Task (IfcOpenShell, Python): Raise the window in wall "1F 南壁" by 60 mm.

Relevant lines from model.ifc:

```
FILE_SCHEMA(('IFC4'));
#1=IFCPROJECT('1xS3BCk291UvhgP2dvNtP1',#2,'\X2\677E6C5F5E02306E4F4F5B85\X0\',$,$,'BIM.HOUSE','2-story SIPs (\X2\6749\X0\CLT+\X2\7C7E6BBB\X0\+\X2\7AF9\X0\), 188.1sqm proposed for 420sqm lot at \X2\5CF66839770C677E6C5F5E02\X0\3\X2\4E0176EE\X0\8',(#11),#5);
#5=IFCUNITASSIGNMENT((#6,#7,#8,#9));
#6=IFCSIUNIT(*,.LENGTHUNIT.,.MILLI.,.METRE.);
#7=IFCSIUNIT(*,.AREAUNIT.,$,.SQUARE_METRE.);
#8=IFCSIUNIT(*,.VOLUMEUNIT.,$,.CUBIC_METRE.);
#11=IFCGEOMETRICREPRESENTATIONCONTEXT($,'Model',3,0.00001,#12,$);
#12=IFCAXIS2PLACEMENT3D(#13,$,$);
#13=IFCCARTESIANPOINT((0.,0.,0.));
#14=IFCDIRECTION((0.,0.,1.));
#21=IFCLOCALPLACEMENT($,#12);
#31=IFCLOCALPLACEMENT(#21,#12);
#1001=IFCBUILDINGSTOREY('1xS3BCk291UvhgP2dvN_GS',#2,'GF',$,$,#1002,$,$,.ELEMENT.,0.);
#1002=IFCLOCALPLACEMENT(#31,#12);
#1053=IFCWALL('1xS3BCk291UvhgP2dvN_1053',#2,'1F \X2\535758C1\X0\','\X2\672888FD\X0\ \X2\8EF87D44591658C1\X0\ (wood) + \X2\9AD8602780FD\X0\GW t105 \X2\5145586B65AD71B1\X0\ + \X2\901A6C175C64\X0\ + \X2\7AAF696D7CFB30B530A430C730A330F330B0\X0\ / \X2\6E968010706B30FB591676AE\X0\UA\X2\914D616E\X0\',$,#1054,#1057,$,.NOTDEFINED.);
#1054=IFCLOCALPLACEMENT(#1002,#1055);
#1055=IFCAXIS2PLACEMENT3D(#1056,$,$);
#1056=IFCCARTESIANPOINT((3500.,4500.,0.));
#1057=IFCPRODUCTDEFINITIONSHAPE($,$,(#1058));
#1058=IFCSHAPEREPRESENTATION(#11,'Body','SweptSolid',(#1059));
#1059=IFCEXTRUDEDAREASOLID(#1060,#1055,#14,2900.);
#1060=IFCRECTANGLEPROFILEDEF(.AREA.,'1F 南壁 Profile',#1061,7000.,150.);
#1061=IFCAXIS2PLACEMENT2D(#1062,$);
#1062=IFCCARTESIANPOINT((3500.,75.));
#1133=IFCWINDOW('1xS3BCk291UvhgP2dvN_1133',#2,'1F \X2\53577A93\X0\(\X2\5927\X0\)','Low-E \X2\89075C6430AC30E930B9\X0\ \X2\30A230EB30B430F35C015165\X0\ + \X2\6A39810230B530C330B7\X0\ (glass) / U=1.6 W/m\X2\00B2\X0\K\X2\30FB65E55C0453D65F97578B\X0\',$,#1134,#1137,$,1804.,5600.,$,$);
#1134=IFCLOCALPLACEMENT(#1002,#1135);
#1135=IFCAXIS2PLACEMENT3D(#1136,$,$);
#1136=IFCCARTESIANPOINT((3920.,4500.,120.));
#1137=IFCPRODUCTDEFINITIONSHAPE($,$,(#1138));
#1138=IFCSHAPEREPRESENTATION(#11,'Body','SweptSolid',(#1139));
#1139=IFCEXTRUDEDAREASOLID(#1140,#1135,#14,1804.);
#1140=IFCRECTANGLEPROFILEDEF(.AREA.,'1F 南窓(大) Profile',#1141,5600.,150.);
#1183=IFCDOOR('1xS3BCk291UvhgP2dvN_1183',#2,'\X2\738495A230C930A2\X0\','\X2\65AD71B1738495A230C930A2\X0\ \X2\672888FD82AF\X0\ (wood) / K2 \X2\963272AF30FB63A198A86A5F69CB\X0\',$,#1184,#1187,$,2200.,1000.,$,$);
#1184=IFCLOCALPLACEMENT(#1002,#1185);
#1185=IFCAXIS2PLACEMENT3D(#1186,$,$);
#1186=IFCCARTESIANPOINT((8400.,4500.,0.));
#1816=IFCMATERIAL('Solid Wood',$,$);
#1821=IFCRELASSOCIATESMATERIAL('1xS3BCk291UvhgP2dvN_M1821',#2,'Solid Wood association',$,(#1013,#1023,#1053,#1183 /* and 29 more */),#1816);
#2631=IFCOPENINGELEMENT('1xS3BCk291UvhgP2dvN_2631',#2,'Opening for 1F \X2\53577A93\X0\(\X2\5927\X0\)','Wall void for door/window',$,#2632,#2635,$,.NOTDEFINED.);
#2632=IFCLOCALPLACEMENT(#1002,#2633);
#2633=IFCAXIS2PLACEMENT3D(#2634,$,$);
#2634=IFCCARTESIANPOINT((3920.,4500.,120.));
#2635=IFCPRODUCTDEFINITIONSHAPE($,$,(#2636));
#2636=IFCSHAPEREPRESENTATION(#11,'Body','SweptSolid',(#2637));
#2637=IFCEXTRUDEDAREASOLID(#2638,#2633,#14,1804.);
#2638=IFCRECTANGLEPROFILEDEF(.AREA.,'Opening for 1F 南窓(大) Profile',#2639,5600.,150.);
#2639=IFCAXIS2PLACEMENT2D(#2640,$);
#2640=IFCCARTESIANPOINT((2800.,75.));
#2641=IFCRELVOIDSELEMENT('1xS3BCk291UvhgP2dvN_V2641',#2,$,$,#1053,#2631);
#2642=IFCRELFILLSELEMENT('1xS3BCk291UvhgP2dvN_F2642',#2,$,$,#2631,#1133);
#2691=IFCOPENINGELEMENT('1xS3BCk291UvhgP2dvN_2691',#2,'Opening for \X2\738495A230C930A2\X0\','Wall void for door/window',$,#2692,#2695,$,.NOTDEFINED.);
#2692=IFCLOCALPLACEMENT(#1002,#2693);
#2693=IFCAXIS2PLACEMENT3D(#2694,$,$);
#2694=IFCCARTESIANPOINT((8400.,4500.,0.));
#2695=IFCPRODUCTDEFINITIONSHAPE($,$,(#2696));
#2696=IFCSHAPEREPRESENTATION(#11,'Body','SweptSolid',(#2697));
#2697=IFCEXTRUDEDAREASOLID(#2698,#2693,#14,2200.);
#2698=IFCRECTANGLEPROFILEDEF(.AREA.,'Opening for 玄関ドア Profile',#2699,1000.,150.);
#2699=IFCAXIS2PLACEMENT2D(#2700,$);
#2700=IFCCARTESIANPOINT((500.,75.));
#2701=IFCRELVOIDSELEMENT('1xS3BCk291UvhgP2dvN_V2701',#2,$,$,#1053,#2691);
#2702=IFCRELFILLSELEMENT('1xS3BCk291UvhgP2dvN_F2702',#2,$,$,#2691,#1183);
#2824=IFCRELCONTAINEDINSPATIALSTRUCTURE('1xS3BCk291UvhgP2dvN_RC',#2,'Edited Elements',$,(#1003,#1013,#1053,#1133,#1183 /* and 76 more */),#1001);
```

```python
import numpy as np
import ifcopenshell
import ifcopenshell.api.geometry
import ifcopenshell.util.placement
import ifcopenshell.util.unit

model = ifcopenshell.open("model.ifc")
unit_scale = ifcopenshell.util.unit.calculate_unit_scale(model)

window = model.by_guid("1xS3BCk291UvhgP2dvN_1133")
opening = window.FillsVoids[0].RelatingOpeningElement
dz = 60.0

shift = np.array([0.0, 0.0, dz])
# The window is not placed relative to its opening, so move both.
for product in (opening, window):
    matrix = ifcopenshell.util.placement.get_local_placement(product.ObjectPlacement)
    matrix[:3, 3] += shift
    ifcopenshell.api.geometry.edit_object_placement(model, product=product, matrix=matrix, is_si=False)

print(f"moved by {dz * unit_scale:+.3f} m")

model.write("model_rev.ifc")
```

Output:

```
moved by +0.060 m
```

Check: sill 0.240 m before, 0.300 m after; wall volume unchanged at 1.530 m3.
